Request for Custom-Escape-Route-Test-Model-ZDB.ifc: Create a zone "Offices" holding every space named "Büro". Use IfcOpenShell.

First a look at what the model holds.

```python
import ifcopenshell

model = ifcopenshell.open("Custom-Escape-Route-Test-Model-ZDB.ifc")
print(model.schema)
seen = {}
for space in model.by_type("IfcSpace"):
    seen[space.LongName] = seen.get(space.LongName, 0) + 1
for name, count in sorted(seen.items(), key=str):
    print(count, "x", name)
print("zones:", [z.Name for z in model.by_type("IfcZone")][:20])
```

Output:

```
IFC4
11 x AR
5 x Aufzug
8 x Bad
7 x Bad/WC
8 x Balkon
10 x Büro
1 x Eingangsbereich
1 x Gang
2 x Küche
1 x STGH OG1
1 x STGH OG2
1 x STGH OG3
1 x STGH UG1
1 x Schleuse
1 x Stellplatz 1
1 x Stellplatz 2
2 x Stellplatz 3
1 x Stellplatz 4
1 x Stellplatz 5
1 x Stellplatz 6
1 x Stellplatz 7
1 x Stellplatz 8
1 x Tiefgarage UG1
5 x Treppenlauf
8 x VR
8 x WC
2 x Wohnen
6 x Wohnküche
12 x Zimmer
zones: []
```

```python
import ifcopenshell
import ifcopenshell.api.group
import ifcopenshell.api.root

model = ifcopenshell.open("Custom-Escape-Route-Test-Model-ZDB.ifc")

names = {"Büro"}
spaces = [s for s in model.by_type("IfcSpace") if s.LongName in names]

zone = ifcopenshell.api.root.create_entity(model, ifc_class="IfcZone", name="Offices")
ifcopenshell.api.group.assign_group(model, products=spaces, group=zone)
print(len(spaces), "spaces in", zone.Name)

model.write("Custom-Escape-Route-Test-Model-ZDB_v2.ifc")
```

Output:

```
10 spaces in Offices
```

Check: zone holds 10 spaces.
